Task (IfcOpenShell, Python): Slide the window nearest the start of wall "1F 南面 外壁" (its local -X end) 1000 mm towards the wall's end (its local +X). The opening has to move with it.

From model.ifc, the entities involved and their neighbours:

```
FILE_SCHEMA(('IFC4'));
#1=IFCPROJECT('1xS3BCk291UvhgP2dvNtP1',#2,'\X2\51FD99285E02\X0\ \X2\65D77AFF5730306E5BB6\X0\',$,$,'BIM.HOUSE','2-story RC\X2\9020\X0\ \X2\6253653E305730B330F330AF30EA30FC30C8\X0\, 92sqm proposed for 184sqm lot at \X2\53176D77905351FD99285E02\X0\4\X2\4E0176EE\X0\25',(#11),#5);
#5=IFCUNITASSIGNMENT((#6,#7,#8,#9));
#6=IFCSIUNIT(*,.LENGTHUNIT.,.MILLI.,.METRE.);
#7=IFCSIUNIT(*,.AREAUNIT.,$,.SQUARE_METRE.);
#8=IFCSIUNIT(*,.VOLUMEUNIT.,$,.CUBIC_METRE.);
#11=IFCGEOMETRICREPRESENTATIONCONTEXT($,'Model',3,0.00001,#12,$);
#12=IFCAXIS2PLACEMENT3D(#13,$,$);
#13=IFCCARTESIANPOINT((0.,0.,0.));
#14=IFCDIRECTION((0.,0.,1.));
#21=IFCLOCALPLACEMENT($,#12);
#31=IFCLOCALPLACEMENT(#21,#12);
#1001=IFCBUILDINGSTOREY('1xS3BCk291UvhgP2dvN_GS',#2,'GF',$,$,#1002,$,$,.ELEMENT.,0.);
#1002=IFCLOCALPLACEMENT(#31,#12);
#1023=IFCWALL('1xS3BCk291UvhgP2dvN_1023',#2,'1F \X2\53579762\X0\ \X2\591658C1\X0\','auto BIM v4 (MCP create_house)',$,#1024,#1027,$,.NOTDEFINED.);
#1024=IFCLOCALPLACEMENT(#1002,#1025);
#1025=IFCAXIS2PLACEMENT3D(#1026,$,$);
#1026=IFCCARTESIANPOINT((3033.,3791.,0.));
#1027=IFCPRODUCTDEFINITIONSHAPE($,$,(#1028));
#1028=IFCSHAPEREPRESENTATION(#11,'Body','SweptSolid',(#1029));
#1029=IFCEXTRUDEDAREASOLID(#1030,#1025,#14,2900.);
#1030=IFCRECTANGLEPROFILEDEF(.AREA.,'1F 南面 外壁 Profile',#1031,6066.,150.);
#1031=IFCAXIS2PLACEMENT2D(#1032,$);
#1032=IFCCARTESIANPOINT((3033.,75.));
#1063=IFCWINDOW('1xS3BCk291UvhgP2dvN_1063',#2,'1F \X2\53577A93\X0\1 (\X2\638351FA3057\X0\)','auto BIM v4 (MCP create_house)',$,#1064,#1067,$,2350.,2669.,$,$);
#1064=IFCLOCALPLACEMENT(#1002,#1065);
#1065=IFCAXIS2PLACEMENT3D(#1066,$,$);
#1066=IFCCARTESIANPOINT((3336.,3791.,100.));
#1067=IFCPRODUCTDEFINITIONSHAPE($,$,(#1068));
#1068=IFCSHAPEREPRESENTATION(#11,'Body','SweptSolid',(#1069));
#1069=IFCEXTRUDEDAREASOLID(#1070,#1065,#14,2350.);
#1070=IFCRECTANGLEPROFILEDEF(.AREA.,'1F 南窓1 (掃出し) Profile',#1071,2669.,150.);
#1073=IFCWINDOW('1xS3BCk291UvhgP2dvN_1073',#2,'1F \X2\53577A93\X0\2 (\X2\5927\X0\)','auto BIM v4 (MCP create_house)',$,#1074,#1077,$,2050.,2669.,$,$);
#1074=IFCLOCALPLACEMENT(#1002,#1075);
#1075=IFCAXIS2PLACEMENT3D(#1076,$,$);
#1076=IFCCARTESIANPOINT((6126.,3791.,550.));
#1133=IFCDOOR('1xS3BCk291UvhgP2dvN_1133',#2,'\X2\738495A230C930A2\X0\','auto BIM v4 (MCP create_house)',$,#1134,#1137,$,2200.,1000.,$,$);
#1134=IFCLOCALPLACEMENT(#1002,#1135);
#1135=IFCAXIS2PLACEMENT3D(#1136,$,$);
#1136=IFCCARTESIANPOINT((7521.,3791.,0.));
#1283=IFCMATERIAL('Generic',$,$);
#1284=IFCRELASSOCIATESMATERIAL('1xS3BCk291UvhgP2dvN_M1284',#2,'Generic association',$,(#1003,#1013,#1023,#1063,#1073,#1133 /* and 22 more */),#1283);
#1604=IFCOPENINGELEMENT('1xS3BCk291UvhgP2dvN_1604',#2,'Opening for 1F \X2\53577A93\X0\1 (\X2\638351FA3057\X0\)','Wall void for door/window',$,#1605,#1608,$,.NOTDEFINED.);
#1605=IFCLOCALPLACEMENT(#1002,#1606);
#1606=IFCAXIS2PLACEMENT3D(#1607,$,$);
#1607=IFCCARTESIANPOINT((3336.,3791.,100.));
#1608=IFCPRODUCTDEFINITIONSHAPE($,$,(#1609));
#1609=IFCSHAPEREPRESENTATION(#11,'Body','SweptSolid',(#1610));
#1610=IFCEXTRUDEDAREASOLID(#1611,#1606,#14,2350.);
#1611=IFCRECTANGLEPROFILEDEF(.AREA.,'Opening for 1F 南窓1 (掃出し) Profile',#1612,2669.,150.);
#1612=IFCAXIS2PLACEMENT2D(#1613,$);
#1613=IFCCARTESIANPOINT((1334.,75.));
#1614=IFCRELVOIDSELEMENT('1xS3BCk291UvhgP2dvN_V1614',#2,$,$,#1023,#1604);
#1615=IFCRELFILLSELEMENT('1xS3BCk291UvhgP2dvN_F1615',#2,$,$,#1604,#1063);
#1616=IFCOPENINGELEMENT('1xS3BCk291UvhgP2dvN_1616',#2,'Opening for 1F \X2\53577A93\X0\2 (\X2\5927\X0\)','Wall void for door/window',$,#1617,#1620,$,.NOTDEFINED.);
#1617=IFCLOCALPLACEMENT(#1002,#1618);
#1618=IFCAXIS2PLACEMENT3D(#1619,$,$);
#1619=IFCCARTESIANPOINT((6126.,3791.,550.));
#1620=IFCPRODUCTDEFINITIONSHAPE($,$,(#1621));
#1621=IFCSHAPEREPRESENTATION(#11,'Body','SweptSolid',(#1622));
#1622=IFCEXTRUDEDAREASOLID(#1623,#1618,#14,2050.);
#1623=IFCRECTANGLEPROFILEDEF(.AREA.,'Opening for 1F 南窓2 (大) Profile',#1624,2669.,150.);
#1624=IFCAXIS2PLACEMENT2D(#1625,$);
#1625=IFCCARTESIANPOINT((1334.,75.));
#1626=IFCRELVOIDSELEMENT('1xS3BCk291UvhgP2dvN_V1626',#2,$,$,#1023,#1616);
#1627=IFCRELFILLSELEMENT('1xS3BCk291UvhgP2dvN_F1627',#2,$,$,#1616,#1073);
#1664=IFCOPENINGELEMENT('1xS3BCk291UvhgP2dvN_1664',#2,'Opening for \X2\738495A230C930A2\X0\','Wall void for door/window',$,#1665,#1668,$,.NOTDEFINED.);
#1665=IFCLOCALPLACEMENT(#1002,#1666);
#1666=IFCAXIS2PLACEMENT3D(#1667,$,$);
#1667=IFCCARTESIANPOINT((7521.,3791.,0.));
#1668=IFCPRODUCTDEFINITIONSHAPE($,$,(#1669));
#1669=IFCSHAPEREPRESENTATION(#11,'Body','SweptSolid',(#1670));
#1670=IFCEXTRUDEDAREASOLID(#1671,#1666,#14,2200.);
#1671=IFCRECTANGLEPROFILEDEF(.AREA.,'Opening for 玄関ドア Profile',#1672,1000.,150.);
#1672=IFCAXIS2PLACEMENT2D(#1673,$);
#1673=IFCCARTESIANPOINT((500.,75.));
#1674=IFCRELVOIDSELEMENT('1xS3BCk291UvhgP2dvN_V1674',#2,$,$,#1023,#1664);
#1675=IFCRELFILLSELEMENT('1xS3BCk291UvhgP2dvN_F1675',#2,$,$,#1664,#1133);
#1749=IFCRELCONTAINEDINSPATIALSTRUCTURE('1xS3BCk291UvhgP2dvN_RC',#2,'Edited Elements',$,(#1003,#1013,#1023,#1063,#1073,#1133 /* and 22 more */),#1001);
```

```python
import ifcopenshell
import ifcopenshell.api.geometry
import ifcopenshell.util.placement
import ifcopenshell.util.unit

model = ifcopenshell.open("model.ifc")
unit_scale = ifcopenshell.util.unit.calculate_unit_scale(model)

window = model.by_id(1063)
opening = window.FillsVoids[0].RelatingOpeningElement
wall = opening.VoidsElements[0].RelatingBuildingElement

wall_matrix = ifcopenshell.util.placement.get_local_placement(wall.ObjectPlacement)
shift = wall_matrix[:3, 0] * 1 / unit_scale
before = ifcopenshell.util.placement.get_local_placement(window.ObjectPlacement)[:3, 3].copy()

# The window is not placed relative to its opening, so move both.
for product in (opening, window):
    matrix = ifcopenshell.util.placement.get_local_placement(product.ObjectPlacement)
    matrix[:3, 3] += shift
    ifcopenshell.api.geometry.edit_object_placement(model, product=product, matrix=matrix, is_si=False)

after = ifcopenshell.util.placement.get_local_placement(window.ObjectPlacement)[:3, 3]
print("window moved by", (after - before).round(3) + 0.0)

model.write("model-out.ifc")
```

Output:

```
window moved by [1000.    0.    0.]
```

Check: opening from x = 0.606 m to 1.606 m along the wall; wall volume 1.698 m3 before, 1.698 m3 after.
